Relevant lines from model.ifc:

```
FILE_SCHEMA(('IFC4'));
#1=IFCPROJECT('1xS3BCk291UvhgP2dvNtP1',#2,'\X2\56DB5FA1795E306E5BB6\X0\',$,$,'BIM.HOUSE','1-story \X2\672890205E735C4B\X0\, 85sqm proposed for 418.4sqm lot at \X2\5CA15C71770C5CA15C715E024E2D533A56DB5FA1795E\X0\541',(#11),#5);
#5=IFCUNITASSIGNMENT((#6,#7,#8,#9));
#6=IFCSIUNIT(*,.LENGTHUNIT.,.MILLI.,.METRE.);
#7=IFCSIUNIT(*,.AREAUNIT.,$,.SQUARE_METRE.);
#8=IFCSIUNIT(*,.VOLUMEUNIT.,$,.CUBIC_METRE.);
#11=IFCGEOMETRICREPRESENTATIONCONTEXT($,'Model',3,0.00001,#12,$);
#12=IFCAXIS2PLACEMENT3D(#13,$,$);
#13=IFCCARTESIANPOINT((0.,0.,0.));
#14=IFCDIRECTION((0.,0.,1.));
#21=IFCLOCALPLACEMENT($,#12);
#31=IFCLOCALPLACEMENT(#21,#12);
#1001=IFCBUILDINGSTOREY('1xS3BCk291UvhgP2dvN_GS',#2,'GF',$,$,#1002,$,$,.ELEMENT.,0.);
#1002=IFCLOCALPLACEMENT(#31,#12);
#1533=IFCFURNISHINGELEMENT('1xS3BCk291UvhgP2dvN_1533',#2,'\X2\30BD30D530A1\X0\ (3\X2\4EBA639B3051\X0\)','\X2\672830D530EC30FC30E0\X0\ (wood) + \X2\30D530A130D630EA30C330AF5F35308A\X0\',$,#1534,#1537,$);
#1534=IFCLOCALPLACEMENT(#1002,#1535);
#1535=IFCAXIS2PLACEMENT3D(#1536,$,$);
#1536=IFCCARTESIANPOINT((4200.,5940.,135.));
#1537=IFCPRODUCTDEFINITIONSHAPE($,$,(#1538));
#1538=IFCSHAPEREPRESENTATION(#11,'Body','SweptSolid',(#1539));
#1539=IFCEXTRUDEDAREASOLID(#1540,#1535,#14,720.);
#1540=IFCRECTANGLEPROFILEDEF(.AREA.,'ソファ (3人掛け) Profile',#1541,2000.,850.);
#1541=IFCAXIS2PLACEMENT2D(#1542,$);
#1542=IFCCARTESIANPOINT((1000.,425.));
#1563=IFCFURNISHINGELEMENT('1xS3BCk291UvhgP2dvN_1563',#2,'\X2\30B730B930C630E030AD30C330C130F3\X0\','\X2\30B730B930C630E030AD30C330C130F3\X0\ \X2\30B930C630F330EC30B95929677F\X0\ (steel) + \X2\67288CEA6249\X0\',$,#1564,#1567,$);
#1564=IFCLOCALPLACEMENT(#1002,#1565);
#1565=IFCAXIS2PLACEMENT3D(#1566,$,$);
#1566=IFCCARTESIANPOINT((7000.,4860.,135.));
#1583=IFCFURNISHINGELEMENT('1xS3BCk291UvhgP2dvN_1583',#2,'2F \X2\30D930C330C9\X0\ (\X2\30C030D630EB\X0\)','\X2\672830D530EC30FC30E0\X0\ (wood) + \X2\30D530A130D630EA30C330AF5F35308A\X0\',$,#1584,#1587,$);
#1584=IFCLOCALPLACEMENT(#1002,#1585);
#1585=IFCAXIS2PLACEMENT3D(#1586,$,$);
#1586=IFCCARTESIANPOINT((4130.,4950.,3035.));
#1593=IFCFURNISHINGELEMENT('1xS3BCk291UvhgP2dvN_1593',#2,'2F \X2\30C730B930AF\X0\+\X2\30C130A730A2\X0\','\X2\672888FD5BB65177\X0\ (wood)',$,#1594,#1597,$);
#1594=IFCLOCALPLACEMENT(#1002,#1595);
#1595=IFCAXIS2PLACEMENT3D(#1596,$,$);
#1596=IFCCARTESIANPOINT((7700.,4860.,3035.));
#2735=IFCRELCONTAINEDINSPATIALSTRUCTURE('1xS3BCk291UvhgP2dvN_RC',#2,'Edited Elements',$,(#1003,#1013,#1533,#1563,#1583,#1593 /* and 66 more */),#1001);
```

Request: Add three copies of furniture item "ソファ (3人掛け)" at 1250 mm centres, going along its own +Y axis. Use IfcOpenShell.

```python
import ifcopenshell
import ifcopenshell.api.geometry
import ifcopenshell.api.root
import ifcopenshell.util.element
import ifcopenshell.util.placement
import ifcopenshell.util.unit

model = ifcopenshell.open("model.ifc")
unit_scale = ifcopenshell.util.unit.calculate_unit_scale(model)


def reuse_history(source, copy):
    """copy_class also copies each property set's owner history, people and application; keep the originals."""
    for rel in copy.IsDefinedBy:
        if rel.is_a("IfcRelDefinesByProperties") and (history := rel.RelatingPropertyDefinition.OwnerHistory):
            rel.RelatingPropertyDefinition.OwnerHistory = source.OwnerHistory
            ifcopenshell.util.element.remove_deep2(model, history)


source = model.by_guid("1xS3BCk291UvhgP2dvN_1533")
base = ifcopenshell.util.placement.get_local_placement(source.ObjectPlacement)
step = base[:3, 1] * 1.25 / unit_scale

for i in range(1, 4):
    copy = ifcopenshell.api.root.copy_class(model, product=source)
    copy.Representation = ifcopenshell.util.element.copy_deep(
        model, source.Representation, exclude=["IfcGeometricRepresentationContext", "IfcRepresentationMap"]
    )
    reuse_history(source, copy)
    matrix = base.copy()
    matrix[:3, 3] += i * step
    print("added at", matrix[:3, 3].round(3) + 0.0)
    ifcopenshell.api.geometry.edit_object_placement(model, product=copy, matrix=matrix, is_si=False)

model.write("model-out.ifc")
```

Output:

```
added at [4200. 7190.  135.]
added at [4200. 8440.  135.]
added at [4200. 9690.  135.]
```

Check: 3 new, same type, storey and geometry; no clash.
